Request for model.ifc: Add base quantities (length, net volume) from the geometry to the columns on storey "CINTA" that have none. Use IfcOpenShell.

First a look at what the model holds.

```python
import ifcopenshell
import ifcopenshell.util.element
import ifcopenshell.util.unit

model = ifcopenshell.open("model.ifc")
print(model.schema)
for unit_type in ("LENGTHUNIT", "AREAUNIT", "VOLUMEUNIT"):
    print(unit_type, ifcopenshell.util.unit.calculate_unit_scale(model, unit_type))
storey = next(s for s in model.by_type("IfcBuildingStorey") if s.Name == "CINTA")
columns = [e for e in ifcopenshell.util.element.get_decomposition(storey) if e.is_a("IfcColumn")]
for e in sorted(columns, key=lambda e: e.id()):
    print(e.id(), e.is_a(), e.Name, list(ifcopenshell.util.element.get_psets(e, qtos_only=True)), sep=" | ")
```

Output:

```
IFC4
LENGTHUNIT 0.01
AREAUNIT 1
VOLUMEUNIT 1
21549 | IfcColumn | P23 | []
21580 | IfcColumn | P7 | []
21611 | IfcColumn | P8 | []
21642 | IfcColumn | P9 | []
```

```python
import ifcopenshell
import ifcopenshell.api.pset
import ifcopenshell.geom
import ifcopenshell.util.element
import ifcopenshell.util.shape
import ifcopenshell.util.unit

model = ifcopenshell.open("model.ifc")
unit_scale = ifcopenshell.util.unit.calculate_unit_scale(model)
volume_scale = ifcopenshell.util.unit.calculate_unit_scale(model, "VOLUMEUNIT")
settings = ifcopenshell.geom.settings()

storey = next(s for s in model.by_type("IfcBuildingStorey") if s.Name == "CINTA")
columns = [e for e in ifcopenshell.util.element.get_decomposition(storey) if e.is_a("IfcColumn")]

for e in sorted(columns, key=lambda e: e.id()):
    if ifcopenshell.util.element.get_psets(e, qtos_only=True, should_inherit=False):
        continue
    # Geometry comes back in metres, in the element's own axes.
    shape = ifcopenshell.geom.create_shape(settings, e)
    values = {
        "Length": ifcopenshell.util.shape.get_z(shape.geometry) / unit_scale,
        "NetVolume": ifcopenshell.util.shape.get_volume(shape.geometry) / volume_scale,
    }
    qto = ifcopenshell.api.pset.add_qto(model, product=e, name="Qto_ColumnBaseQuantities")
    ifcopenshell.api.pset.edit_qto(model, qto=qto, properties=values)
    print(e.id(), {k: round(v, 3) for k, v in values.items()})

model.write("model-out.ifc")
```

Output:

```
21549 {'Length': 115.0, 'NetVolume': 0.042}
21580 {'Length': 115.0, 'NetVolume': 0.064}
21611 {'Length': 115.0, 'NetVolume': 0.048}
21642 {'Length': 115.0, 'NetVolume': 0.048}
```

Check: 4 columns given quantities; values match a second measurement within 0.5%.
